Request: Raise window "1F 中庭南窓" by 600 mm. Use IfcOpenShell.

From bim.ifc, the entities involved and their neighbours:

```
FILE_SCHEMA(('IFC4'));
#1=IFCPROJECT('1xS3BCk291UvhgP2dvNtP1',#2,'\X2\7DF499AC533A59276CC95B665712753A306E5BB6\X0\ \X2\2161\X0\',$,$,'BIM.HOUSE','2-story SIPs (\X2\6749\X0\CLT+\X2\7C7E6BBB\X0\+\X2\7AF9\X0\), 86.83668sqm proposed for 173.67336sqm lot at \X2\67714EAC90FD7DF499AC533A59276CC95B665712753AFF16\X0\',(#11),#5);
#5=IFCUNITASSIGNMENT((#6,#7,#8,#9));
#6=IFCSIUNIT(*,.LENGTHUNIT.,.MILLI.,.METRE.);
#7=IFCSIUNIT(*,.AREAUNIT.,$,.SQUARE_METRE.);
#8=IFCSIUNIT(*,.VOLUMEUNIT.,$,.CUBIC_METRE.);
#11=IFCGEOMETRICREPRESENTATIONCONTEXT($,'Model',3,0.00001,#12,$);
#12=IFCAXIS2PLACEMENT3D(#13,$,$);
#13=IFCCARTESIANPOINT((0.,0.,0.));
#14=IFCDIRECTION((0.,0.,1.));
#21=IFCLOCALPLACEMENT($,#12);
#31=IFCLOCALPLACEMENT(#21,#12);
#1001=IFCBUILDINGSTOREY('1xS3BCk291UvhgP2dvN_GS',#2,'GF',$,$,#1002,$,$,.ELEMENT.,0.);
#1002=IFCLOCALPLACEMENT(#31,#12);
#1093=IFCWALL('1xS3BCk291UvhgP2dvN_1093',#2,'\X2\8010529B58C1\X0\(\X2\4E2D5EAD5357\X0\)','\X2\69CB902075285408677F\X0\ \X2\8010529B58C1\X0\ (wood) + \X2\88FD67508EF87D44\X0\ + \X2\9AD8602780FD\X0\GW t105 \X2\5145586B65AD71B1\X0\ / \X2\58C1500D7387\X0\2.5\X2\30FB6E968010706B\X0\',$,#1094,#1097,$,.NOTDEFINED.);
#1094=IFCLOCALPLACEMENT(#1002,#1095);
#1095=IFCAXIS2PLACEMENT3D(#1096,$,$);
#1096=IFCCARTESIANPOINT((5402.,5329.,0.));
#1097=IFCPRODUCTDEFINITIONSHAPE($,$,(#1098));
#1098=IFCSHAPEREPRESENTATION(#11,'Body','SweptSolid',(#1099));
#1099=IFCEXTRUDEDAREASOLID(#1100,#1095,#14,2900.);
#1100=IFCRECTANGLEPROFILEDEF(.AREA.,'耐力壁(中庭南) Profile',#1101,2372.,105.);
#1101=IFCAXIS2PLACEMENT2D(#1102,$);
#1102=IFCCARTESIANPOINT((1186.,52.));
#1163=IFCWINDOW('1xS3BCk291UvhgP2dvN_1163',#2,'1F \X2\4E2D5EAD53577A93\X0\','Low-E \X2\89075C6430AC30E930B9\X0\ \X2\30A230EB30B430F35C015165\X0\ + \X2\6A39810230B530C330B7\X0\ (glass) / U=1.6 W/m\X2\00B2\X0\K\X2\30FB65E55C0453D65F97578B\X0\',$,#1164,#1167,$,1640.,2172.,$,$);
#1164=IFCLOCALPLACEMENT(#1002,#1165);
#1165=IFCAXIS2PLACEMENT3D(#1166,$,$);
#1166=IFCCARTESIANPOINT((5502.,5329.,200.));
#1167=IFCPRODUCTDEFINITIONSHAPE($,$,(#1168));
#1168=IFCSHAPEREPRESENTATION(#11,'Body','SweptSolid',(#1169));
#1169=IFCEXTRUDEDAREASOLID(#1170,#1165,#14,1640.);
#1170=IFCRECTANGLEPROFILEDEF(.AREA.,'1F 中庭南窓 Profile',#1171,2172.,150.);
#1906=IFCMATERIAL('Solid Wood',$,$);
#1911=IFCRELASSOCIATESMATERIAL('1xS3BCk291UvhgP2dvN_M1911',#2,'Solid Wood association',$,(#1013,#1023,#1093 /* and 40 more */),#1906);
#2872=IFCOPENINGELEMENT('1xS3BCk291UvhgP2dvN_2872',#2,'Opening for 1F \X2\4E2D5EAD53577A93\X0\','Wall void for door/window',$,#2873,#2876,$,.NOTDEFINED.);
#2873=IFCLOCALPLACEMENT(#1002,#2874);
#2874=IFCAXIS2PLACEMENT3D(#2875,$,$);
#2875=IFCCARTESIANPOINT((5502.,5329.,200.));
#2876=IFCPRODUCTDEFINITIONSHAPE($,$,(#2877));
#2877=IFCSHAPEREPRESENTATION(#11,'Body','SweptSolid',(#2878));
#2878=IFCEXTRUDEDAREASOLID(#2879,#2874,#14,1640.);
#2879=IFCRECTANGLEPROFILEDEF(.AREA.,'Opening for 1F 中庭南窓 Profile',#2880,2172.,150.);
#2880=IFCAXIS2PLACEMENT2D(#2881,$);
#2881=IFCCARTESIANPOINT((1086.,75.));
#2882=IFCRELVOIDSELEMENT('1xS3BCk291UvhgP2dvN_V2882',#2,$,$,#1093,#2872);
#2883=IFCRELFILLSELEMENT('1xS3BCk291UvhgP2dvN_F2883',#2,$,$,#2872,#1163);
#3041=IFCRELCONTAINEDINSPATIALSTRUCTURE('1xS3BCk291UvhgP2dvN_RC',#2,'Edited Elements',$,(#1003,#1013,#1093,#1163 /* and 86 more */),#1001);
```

```python
import numpy as np
import ifcopenshell
import ifcopenshell.api.geometry
import ifcopenshell.util.placement
import ifcopenshell.util.unit

model = ifcopenshell.open("bim.ifc")
unit_scale = ifcopenshell.util.unit.calculate_unit_scale(model)

window = model.by_id(1163)
opening = window.FillsVoids[0].RelatingOpeningElement
dz = 600.0

shift = np.array([0.0, 0.0, dz])
# The window is not placed relative to its opening, so move both.
for product in (opening, window):
    matrix = ifcopenshell.util.placement.get_local_placement(product.ObjectPlacement)
    matrix[:3, 3] += shift
    ifcopenshell.api.geometry.edit_object_placement(model, product=product, matrix=matrix, is_si=False)

print(f"moved by {dz * unit_scale:+.3f} m")

model.write("bim_edited.ifc")
```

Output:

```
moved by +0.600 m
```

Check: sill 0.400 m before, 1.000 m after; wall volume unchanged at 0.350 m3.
